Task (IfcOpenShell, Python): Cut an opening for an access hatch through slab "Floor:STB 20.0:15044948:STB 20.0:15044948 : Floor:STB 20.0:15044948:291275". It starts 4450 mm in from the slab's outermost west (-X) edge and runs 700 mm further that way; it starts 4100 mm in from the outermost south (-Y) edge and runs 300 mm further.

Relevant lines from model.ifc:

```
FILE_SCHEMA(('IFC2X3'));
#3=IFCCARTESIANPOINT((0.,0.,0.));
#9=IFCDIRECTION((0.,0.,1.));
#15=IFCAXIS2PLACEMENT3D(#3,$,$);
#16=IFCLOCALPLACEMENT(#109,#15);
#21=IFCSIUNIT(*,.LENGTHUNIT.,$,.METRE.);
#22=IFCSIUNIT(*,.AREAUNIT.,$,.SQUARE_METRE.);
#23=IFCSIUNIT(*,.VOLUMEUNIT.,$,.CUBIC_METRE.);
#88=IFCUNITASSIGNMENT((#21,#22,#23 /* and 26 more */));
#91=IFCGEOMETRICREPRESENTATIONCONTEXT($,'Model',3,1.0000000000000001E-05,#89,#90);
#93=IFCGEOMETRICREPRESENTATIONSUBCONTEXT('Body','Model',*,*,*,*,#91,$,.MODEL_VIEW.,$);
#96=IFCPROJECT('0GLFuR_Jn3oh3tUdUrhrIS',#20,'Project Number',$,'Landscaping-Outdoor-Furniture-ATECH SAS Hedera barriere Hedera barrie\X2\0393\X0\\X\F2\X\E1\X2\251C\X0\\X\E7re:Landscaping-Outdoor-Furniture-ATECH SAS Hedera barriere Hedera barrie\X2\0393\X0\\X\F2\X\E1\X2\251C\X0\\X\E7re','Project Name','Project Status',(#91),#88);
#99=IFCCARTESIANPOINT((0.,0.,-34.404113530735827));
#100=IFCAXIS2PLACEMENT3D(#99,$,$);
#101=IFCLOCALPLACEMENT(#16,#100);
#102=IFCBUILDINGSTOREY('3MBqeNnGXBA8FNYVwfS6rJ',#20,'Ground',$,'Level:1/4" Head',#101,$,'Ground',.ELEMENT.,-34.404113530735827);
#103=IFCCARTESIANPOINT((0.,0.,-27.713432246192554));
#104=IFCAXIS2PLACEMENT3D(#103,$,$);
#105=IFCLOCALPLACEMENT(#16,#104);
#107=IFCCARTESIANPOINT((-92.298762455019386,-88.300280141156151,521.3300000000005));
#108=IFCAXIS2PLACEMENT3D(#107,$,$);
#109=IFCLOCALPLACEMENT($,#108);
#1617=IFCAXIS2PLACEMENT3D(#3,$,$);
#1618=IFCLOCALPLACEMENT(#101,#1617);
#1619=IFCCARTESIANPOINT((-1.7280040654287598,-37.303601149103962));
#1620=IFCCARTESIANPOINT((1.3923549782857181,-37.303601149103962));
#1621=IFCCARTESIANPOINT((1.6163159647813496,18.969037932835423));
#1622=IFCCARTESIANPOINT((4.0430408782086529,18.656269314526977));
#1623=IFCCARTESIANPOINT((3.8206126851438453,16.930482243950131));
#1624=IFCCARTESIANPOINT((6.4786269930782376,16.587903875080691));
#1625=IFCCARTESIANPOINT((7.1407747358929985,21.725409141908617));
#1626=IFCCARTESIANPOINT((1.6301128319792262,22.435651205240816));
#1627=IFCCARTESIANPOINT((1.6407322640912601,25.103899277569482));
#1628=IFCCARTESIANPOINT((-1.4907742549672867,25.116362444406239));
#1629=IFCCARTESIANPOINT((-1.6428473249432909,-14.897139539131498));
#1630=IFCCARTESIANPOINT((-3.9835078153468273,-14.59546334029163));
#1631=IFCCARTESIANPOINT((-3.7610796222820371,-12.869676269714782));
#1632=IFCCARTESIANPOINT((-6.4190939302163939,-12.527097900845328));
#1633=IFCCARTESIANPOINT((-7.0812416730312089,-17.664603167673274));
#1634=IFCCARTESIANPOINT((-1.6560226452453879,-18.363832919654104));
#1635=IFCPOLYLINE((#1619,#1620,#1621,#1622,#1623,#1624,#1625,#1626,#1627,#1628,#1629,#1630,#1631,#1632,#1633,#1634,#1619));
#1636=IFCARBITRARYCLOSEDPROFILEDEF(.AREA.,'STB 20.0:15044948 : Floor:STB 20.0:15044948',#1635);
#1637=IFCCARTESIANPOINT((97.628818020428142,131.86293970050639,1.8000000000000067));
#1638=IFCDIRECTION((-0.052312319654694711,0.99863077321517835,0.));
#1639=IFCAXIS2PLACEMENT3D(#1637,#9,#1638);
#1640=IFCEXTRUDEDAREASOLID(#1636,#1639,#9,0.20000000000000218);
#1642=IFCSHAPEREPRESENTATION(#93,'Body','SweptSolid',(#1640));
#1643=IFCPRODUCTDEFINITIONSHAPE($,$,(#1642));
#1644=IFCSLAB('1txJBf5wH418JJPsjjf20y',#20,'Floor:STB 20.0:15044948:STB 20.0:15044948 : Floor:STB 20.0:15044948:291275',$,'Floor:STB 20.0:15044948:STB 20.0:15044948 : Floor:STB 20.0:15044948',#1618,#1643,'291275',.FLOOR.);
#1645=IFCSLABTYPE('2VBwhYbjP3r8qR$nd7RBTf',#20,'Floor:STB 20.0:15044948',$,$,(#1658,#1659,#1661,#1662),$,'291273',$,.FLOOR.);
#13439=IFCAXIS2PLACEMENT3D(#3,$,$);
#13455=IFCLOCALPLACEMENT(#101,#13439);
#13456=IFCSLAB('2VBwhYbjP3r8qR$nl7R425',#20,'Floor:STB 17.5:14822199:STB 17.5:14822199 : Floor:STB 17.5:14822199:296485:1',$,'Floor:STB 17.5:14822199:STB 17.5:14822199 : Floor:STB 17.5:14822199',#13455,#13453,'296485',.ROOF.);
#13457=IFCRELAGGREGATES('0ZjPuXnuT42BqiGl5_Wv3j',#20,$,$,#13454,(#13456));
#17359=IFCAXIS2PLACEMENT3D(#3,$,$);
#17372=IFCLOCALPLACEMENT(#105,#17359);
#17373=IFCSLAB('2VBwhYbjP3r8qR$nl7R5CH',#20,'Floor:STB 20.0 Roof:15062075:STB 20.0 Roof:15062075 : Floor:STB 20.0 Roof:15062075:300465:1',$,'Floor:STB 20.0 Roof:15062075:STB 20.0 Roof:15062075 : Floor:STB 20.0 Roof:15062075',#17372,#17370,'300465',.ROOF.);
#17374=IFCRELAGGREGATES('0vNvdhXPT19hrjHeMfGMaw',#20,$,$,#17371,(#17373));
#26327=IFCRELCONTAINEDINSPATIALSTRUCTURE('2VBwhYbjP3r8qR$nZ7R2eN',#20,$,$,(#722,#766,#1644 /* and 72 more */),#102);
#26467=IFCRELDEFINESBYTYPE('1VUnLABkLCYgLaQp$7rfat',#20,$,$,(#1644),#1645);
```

```python
import numpy as np
import ifcopenshell
import ifcopenshell.api.feature
import ifcopenshell.api.geometry
import ifcopenshell.api.root
import ifcopenshell.geom
import ifcopenshell.util.placement
import ifcopenshell.util.representation
import ifcopenshell.util.shape
import ifcopenshell.util.unit

model = ifcopenshell.open("model.ifc")
unit_scale = ifcopenshell.util.unit.calculate_unit_scale(model)
settings = ifcopenshell.geom.settings()


def volume(element):
    """Net volume in cubic metres, openings subtracted."""
    shape = ifcopenshell.geom.create_shape(settings, element)
    return ifcopenshell.util.shape.get_volume(shape.geometry)


slab = model.by_guid("1txJBf5wH418JJPsjjf20y")
before = volume(slab)

# Extent in the slab's own axes, in metres. The edges named are its -X and -Y sides.
slab_shape = ifcopenshell.geom.create_shape(settings, slab)
vertices = ifcopenshell.util.shape.get_vertices(slab_shape.geometry)
x_min, y_min, bottom = vertices.min(axis=0)
top = vertices[:, 2].max()

opening = ifcopenshell.api.root.create_entity(model, ifc_class="IfcOpeningElement", name="Access hatch opening")
context = ifcopenshell.util.representation.get_context(model, "Model", "Body", "MODEL_VIEW")
width, depth = 0.7, 0.3
outline = [(0.0, 0.0), (width, 0.0), (width, depth), (0.0, depth), (0.0, 0.0)]
# Overshoot both faces by 50 mm so the cut is clean.
shape = ifcopenshell.api.geometry.add_slab_representation(
    model, context=context, depth=top - bottom + 0.1, polyline=outline
)
ifcopenshell.api.geometry.assign_representation(model, product=opening, representation=shape)

matrix = ifcopenshell.util.placement.get_local_placement(slab.ObjectPlacement)
matrix[:, 3] = matrix @ np.append(np.array([x_min + 4.45, y_min + 4.1, bottom - 0.05]) / unit_scale, 1.0)
ifcopenshell.api.geometry.edit_object_placement(model, product=opening, matrix=matrix, is_si=False)
ifcopenshell.api.feature.add_feature(model, feature=opening, element=slab)

after = volume(slab)

print(f"slab volume {before:.3f} -> {after:.3f} m3")

model.write("model-out.ifc")
```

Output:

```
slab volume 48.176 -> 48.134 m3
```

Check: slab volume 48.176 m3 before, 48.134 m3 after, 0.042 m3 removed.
